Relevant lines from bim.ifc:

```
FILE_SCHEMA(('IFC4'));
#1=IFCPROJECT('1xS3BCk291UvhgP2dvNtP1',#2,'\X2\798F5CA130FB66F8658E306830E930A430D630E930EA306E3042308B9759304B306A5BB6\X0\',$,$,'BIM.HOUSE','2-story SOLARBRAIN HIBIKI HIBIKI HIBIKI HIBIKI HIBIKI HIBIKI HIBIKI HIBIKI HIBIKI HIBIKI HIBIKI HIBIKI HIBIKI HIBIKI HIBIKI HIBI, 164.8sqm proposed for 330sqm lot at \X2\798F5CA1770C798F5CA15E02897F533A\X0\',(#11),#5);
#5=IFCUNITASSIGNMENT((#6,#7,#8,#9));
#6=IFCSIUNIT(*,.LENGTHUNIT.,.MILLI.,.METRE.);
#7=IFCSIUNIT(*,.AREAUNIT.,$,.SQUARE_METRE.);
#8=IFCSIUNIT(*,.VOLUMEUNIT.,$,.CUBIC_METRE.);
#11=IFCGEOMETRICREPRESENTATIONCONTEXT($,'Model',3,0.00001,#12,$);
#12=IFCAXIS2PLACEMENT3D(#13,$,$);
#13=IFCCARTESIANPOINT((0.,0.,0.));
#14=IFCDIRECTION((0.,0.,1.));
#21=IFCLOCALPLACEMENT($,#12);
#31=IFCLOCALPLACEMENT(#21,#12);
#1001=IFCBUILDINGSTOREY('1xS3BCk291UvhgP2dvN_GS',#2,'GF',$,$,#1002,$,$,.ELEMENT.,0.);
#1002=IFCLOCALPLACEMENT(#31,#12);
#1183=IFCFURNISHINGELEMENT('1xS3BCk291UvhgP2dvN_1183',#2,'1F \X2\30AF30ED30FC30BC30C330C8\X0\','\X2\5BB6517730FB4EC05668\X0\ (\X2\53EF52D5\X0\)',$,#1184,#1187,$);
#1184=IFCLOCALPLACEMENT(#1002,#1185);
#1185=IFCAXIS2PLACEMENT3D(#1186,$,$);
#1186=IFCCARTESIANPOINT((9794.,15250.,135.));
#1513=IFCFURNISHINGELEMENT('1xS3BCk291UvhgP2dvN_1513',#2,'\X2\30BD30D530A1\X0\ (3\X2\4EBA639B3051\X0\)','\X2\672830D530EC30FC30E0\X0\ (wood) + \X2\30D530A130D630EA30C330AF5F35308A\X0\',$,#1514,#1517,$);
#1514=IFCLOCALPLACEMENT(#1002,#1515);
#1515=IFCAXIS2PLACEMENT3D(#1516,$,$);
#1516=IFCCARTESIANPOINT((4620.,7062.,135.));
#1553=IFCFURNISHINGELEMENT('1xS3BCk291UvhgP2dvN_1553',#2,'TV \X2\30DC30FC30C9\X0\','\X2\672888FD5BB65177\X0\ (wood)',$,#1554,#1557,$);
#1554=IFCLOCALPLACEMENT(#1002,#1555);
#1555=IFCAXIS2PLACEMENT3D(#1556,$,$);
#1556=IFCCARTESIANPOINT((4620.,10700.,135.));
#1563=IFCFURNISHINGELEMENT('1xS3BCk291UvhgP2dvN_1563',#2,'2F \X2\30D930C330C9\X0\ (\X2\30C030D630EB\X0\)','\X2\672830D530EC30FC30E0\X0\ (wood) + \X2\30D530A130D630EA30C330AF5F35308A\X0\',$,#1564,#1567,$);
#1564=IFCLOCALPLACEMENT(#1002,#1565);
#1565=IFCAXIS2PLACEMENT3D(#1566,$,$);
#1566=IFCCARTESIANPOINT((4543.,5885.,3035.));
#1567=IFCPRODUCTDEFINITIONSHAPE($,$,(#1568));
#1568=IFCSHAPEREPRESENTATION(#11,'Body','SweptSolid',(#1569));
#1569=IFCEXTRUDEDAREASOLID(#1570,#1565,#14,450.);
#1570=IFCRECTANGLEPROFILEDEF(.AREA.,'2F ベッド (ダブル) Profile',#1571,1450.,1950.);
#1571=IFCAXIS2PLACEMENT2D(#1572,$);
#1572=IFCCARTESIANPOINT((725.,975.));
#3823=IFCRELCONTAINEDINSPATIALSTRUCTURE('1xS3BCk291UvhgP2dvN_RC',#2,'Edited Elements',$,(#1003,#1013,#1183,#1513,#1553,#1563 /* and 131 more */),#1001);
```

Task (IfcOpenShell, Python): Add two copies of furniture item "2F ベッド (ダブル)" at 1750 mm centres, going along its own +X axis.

```python
import ifcopenshell
import ifcopenshell.api.geometry
import ifcopenshell.api.root
import ifcopenshell.util.element
import ifcopenshell.util.placement
import ifcopenshell.util.unit

model = ifcopenshell.open("bim.ifc")
unit_scale = ifcopenshell.util.unit.calculate_unit_scale(model)


def reuse_history(source, copy):
    """copy_class also copies each property set's owner history, people and application; keep the originals."""
    for rel in copy.IsDefinedBy:
        if rel.is_a("IfcRelDefinesByProperties") and (history := rel.RelatingPropertyDefinition.OwnerHistory):
            rel.RelatingPropertyDefinition.OwnerHistory = source.OwnerHistory
            ifcopenshell.util.element.remove_deep2(model, history)


source = model.by_guid("1xS3BCk291UvhgP2dvN_1563")
base = ifcopenshell.util.placement.get_local_placement(source.ObjectPlacement)
step = base[:3, 0] * 1.75 / unit_scale

for i in range(1, 3):
    copy = ifcopenshell.api.root.copy_class(model, product=source)
    copy.Representation = ifcopenshell.util.element.copy_deep(
        model, source.Representation, exclude=["IfcGeometricRepresentationContext", "IfcRepresentationMap"]
    )
    reuse_history(source, copy)
    matrix = base.copy()
    matrix[:3, 3] += i * step
    print("added at", matrix[:3, 3].round(3) + 0.0)
    ifcopenshell.api.geometry.edit_object_placement(model, product=copy, matrix=matrix, is_si=False)

model.write("bim_edited.ifc")
```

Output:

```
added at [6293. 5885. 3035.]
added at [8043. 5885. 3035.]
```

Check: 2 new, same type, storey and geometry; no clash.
